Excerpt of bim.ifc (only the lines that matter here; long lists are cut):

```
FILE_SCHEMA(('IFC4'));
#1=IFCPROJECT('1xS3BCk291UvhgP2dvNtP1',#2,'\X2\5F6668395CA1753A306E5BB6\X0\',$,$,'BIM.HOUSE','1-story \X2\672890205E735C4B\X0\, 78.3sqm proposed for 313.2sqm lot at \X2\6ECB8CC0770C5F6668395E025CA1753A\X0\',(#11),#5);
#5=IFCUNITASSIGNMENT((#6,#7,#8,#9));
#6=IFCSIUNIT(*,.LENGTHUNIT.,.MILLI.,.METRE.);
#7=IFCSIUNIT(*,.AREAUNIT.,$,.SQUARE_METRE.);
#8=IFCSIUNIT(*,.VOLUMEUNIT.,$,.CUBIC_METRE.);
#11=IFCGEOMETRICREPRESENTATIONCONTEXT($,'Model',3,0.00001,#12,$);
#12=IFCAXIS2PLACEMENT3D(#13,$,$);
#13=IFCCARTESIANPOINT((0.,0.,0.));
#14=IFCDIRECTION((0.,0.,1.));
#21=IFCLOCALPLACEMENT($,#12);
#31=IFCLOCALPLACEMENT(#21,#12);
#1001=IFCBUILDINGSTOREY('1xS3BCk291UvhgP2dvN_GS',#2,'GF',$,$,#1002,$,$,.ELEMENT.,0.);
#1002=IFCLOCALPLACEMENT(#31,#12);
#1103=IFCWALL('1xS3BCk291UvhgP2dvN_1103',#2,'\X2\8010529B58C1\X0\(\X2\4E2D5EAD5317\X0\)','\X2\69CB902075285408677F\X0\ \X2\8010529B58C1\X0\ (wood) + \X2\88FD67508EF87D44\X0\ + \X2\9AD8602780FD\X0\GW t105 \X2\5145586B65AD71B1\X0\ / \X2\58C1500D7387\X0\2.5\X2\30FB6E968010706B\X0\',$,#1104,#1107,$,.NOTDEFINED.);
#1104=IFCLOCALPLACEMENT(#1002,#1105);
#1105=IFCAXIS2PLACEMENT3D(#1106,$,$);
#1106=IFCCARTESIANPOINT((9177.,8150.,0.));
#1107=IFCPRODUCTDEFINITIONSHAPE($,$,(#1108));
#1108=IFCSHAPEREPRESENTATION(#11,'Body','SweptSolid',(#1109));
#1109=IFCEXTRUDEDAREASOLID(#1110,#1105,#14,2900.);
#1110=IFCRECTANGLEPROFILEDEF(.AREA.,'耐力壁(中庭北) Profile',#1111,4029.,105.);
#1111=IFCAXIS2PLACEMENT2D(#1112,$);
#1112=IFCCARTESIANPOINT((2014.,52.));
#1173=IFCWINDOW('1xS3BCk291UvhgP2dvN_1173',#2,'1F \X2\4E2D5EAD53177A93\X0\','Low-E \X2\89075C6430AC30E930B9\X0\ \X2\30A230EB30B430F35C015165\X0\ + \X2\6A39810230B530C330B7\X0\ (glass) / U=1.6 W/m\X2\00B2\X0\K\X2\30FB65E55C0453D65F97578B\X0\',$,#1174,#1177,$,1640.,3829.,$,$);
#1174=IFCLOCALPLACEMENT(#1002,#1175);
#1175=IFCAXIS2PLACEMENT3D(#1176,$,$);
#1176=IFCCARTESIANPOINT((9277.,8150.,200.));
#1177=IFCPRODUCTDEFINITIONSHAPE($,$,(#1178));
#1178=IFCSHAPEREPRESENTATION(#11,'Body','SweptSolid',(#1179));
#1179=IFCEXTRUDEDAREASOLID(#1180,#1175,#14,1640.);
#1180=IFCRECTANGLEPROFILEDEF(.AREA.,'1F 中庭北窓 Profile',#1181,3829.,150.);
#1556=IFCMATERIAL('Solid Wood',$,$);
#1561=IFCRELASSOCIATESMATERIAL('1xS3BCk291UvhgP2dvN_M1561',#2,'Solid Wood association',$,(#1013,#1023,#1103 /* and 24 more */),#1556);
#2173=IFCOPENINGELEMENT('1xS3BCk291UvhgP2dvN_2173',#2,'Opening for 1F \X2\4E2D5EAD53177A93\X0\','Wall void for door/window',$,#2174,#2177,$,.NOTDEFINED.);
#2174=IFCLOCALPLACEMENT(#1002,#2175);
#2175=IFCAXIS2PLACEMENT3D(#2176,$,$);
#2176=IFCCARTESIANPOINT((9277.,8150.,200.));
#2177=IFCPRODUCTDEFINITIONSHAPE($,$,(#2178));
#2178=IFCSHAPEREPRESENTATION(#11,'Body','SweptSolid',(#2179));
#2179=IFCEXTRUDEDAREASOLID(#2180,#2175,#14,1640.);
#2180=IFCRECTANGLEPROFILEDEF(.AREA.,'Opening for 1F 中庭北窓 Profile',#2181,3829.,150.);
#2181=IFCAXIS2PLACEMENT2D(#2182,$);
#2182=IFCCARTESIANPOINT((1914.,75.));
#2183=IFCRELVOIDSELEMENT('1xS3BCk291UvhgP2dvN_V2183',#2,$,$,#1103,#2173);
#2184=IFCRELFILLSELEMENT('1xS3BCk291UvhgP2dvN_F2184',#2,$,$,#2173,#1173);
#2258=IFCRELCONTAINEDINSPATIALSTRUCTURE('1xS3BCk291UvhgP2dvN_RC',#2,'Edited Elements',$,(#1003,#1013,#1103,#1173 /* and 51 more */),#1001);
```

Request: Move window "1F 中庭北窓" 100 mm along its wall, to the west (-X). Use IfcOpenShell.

```python
import ifcopenshell
import ifcopenshell.api.geometry
import ifcopenshell.util.placement
import ifcopenshell.util.unit

model = ifcopenshell.open("bim.ifc")
unit_scale = ifcopenshell.util.unit.calculate_unit_scale(model)

window = model.by_guid("1xS3BCk291UvhgP2dvN_1173")
opening = window.FillsVoids[0].RelatingOpeningElement
wall = opening.VoidsElements[0].RelatingBuildingElement

wall_matrix = ifcopenshell.util.placement.get_local_placement(wall.ObjectPlacement)
shift = wall_matrix[:3, 0] * -0.1 / unit_scale
before = ifcopenshell.util.placement.get_local_placement(window.ObjectPlacement)[:3, 3].copy()

# The window is not placed relative to its opening, so move both.
for product in (opening, window):
    matrix = ifcopenshell.util.placement.get_local_placement(product.ObjectPlacement)
    matrix[:3, 3] += shift
    ifcopenshell.api.geometry.edit_object_placement(model, product=product, matrix=matrix, is_si=False)

after = ifcopenshell.util.placement.get_local_placement(window.ObjectPlacement)[:3, 3]
print("window moved by", (after - before).round(3) + 0.0)

model.write("bim_edited.ifc")
```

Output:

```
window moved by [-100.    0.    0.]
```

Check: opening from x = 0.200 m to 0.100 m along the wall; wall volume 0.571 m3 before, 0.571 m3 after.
